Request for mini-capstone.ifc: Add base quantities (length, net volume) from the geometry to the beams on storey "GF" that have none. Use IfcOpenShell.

First a look at what the model holds.

```python
import ifcopenshell
import ifcopenshell.util.element
import ifcopenshell.util.unit

model = ifcopenshell.open("mini-capstone.ifc")
print(model.schema)
for unit_type in ("LENGTHUNIT", "AREAUNIT", "VOLUMEUNIT"):
    print(unit_type, ifcopenshell.util.unit.calculate_unit_scale(model, unit_type))
storey = next(s for s in model.by_type("IfcBuildingStorey") if s.Name == "GF")
beams = [e for e in ifcopenshell.util.element.get_decomposition(storey) if e.is_a("IfcBeam")]
for e in sorted(beams, key=lambda e: e.id()):
    print(e.id(), e.is_a(), e.Name, list(ifcopenshell.util.element.get_psets(e, qtos_only=True)), sep=" | ")
```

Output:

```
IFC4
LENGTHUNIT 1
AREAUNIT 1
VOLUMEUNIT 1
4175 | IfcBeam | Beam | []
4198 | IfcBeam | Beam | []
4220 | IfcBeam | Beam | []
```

```python
import ifcopenshell
import ifcopenshell.api.pset
import ifcopenshell.geom
import ifcopenshell.util.element
import ifcopenshell.util.shape
import ifcopenshell.util.unit

model = ifcopenshell.open("mini-capstone.ifc")
unit_scale = ifcopenshell.util.unit.calculate_unit_scale(model)
volume_scale = ifcopenshell.util.unit.calculate_unit_scale(model, "VOLUMEUNIT")
settings = ifcopenshell.geom.settings()

storey = next(s for s in model.by_type("IfcBuildingStorey") if s.Name == "GF")
beams = [e for e in ifcopenshell.util.element.get_decomposition(storey) if e.is_a("IfcBeam")]

for e in sorted(beams, key=lambda e: e.id()):
    if ifcopenshell.util.element.get_psets(e, qtos_only=True, should_inherit=False):
        continue
    # Geometry comes back in metres, in the element's own axes.
    shape = ifcopenshell.geom.create_shape(settings, e)
    values = {
        "Length": ifcopenshell.util.shape.get_max_xyz(shape.geometry) / unit_scale,
        "NetVolume": ifcopenshell.util.shape.get_volume(shape.geometry) / volume_scale,
    }
    qto = ifcopenshell.api.pset.add_qto(model, product=e, name="Qto_BeamBaseQuantities")
    ifcopenshell.api.pset.edit_qto(model, qto=qto, properties=values)
    print(e.id(), {k: round(v, 3) for k, v in values.items()})

model.write("mini-capstone_v2.ifc")
```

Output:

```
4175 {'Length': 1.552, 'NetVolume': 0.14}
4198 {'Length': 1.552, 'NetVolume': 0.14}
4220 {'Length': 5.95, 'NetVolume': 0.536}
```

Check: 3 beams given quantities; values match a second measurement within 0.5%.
